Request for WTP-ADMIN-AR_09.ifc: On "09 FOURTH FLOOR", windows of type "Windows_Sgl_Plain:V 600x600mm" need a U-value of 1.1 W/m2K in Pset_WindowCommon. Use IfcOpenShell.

First a look at what the model holds.

```python
import ifcopenshell
import ifcopenshell.util.element

model = ifcopenshell.open("WTP-ADMIN-AR_09.ifc")
print(model.schema)
storey = next(s for s in model.by_type("IfcBuildingStorey") if s.Name == "09 FOURTH FLOOR")
windows = [e for e in ifcopenshell.util.element.get_decomposition(storey) if e.is_a("IfcWindow")]
seen = {}
for e in windows:
    element_type = ifcopenshell.util.element.get_type(e)
    key = (element_type.Name if element_type != e and element_type else None, ifcopenshell.util.element.get_pset(e, "Pset_WindowCommon", "ThermalTransmittance"))
    seen[key] = seen.get(key, 0) + 1
for (name, value), count in sorted(seen.items(), key=str):
    print(count, "x", name, "|", value)
```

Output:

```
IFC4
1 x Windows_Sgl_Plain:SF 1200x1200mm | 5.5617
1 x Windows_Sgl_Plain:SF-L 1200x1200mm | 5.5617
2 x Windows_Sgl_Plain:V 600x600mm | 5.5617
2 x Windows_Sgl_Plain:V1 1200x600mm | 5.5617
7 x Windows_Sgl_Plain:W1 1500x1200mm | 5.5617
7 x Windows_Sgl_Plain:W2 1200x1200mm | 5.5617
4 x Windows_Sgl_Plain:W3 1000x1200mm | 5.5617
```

```python
import ifcopenshell
import ifcopenshell.api.pset
import ifcopenshell.util.element

model = ifcopenshell.open("WTP-ADMIN-AR_09.ifc")

storey = next(s for s in model.by_type("IfcBuildingStorey") if s.Name == "09 FOURTH FLOOR")
windows = [e for e in ifcopenshell.util.element.get_decomposition(storey) if e.is_a("IfcWindow")]

count = 0
for e in windows:
    element_type = ifcopenshell.util.element.get_type(e)
    if element_type in (None, e) or element_type.Name != "Windows_Sgl_Plain:V 600x600mm":
        continue
    # add_pset returns the element's existing set when there is one.
    pset = ifcopenshell.api.pset.add_pset(model, product=e, name="Pset_WindowCommon")
    ifcopenshell.api.pset.edit_pset(model, pset=pset, properties={"ThermalTransmittance": 1.1})
    count += 1

print(count, "windows updated")

model.write("WTP-ADMIN-AR_09_v2.ifc")
```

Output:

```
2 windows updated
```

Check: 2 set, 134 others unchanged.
